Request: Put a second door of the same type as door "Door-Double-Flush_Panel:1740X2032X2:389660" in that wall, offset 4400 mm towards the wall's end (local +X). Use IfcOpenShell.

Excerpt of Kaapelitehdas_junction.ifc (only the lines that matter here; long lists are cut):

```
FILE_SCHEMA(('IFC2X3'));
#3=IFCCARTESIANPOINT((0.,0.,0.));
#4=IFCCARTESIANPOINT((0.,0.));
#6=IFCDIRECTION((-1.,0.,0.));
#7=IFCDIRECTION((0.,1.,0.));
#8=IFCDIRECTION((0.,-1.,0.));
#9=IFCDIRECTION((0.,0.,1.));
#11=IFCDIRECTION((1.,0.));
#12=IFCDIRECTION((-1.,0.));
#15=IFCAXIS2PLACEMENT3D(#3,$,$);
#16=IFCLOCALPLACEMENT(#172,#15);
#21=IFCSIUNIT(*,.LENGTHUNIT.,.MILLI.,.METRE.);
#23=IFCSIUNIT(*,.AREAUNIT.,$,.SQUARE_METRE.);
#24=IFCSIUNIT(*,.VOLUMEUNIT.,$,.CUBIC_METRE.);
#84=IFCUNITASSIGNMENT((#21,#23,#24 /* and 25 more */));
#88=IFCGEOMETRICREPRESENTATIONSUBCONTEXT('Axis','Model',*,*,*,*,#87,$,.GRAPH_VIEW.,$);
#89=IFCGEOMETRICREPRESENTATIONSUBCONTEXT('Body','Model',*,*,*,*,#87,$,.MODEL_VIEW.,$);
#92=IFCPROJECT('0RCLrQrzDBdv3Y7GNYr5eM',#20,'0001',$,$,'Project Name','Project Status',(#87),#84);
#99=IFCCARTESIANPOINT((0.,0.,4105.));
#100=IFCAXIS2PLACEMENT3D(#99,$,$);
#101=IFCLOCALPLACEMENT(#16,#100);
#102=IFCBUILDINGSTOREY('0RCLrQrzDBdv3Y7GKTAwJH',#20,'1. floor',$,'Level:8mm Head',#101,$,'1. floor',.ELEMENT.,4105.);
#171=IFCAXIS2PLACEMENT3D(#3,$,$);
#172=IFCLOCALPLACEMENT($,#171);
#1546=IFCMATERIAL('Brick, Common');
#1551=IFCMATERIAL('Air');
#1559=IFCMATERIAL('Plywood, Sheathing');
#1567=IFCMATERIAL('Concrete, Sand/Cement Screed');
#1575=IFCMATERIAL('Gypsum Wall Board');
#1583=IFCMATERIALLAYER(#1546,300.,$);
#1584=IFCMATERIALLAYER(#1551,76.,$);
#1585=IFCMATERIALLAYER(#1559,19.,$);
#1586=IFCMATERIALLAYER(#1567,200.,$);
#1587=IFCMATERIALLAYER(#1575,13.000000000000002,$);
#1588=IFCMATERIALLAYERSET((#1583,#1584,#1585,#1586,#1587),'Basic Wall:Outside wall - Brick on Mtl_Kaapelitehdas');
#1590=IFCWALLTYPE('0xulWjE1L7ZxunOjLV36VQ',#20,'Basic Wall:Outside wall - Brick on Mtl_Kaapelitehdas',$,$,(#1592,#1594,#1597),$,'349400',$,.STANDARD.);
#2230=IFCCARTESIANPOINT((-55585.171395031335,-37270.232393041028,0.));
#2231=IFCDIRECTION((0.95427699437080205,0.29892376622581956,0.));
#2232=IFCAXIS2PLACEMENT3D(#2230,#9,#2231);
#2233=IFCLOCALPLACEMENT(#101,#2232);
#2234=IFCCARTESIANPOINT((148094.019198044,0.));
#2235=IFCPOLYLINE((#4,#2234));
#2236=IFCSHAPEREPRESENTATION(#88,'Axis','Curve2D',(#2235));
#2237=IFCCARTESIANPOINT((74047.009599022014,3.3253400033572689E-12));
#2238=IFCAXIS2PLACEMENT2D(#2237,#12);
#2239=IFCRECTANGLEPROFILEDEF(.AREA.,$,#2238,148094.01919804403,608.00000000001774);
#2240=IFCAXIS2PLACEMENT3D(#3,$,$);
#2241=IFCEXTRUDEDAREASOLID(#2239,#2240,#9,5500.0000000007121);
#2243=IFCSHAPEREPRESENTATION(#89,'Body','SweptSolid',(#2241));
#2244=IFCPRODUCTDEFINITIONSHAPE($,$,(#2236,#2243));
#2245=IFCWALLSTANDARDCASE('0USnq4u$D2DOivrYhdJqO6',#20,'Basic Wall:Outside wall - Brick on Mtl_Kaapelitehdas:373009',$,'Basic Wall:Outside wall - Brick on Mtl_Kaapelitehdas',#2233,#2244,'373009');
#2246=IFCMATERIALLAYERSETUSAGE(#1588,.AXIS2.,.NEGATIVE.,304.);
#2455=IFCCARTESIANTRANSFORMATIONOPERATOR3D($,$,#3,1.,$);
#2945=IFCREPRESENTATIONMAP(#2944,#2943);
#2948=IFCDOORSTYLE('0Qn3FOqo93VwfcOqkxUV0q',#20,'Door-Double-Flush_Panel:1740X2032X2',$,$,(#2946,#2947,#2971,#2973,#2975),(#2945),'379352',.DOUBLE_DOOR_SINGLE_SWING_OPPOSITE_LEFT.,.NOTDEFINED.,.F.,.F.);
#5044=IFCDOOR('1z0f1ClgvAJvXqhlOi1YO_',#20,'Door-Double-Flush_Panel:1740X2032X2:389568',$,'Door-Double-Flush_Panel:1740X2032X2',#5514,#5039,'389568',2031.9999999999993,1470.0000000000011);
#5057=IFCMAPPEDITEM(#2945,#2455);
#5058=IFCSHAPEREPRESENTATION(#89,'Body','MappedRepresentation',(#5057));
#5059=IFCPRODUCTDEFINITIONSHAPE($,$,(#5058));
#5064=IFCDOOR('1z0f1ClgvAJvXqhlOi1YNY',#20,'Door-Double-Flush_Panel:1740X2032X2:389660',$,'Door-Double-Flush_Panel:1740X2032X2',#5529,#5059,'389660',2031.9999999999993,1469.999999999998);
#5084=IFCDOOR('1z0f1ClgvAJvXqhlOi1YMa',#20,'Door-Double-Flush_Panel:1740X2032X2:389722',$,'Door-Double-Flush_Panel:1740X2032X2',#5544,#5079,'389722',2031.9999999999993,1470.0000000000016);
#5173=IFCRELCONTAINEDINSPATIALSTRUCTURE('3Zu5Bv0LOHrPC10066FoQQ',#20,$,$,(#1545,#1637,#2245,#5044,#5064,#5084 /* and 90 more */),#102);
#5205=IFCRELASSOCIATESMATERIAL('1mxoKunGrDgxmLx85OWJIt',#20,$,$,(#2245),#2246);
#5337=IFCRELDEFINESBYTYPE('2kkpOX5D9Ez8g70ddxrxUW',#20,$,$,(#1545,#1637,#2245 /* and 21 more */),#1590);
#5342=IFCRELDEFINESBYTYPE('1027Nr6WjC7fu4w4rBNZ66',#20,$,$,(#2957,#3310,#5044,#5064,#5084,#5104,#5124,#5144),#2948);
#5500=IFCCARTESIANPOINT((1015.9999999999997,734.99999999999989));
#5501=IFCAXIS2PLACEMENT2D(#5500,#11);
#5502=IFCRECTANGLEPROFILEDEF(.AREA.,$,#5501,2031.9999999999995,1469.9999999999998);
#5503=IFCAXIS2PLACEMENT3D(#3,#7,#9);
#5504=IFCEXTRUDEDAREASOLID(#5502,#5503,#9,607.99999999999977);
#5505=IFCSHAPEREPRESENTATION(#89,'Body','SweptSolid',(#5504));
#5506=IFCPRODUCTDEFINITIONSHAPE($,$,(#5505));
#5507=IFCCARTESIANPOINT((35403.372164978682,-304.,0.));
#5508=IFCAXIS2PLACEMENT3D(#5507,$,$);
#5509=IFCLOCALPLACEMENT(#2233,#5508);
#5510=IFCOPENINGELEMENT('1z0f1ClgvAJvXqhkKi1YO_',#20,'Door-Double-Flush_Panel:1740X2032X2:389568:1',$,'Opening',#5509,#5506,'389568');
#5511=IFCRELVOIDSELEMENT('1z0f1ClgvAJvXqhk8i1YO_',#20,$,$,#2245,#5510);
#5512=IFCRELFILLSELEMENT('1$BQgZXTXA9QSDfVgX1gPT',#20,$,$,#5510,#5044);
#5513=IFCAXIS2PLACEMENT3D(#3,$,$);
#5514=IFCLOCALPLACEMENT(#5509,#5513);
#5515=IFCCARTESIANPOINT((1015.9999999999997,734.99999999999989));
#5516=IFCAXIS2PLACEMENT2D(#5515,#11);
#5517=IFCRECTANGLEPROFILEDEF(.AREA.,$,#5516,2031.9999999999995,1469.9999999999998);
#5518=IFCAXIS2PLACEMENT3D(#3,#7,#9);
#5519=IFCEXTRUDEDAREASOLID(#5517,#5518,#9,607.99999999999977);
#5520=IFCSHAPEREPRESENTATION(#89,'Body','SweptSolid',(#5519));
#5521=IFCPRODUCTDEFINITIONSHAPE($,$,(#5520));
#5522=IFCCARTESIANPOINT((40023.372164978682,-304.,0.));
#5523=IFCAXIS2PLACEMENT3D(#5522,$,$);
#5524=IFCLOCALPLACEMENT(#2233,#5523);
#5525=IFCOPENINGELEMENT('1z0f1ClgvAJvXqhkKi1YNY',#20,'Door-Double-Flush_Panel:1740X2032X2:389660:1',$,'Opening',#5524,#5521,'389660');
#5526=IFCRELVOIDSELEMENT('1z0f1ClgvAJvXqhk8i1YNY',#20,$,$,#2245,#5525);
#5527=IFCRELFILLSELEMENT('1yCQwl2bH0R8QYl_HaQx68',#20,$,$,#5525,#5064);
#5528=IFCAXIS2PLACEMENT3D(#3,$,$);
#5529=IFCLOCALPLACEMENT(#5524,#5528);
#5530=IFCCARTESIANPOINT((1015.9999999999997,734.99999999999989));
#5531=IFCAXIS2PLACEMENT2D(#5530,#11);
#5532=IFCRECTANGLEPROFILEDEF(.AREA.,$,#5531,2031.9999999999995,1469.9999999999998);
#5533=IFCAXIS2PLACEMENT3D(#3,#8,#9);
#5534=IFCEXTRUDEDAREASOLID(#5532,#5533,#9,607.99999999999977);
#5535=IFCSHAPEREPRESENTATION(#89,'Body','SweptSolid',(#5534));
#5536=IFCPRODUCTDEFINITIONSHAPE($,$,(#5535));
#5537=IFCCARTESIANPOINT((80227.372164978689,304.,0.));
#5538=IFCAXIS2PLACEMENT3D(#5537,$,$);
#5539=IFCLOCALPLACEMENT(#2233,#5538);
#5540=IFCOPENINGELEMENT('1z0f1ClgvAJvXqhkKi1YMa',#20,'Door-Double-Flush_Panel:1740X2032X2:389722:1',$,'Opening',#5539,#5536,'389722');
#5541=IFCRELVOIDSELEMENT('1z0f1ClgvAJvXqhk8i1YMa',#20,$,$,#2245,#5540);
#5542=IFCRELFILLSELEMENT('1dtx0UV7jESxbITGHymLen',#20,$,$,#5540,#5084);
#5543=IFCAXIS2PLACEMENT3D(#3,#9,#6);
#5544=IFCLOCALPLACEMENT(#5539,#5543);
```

```python
import ifcopenshell
import ifcopenshell.api.feature
import ifcopenshell.api.geometry
import ifcopenshell.api.root
import ifcopenshell.geom
import ifcopenshell.util.element
import ifcopenshell.util.placement
import ifcopenshell.util.shape

model = ifcopenshell.open("Kaapelitehdas_junction.ifc")
settings = ifcopenshell.geom.settings()


def volume(element):
    """Net volume in cubic metres, openings subtracted."""
    shape = ifcopenshell.geom.create_shape(settings, element)
    return ifcopenshell.util.shape.get_volume(shape.geometry)


def reuse_history(source, copy):
    """copy_class also copies each property set's owner history, people and application; keep the originals."""
    for rel in copy.IsDefinedBy:
        if rel.is_a("IfcRelDefinesByProperties") and (history := rel.RelatingPropertyDefinition.OwnerHistory):
            rel.RelatingPropertyDefinition.OwnerHistory = source.OwnerHistory
            ifcopenshell.util.element.remove_deep2(model, history)


door = model.by_id(5064)
opening = door.FillsVoids[0].RelatingOpeningElement
wall = opening.VoidsElements[0].RelatingBuildingElement
before = volume(wall)
shift = ifcopenshell.util.placement.get_local_placement(wall.ObjectPlacement)[:3, 0] * 4400.0

# copy_class copies the void relationship, type, container and properties, but no geometry.
new_opening = ifcopenshell.api.root.copy_class(model, product=opening)
new_opening.Representation = ifcopenshell.util.element.copy_deep(
    model, opening.Representation, exclude=["IfcGeometricRepresentationContext", "IfcRepresentationMap"]
)
new_opening.Name = "Door-Double-Flush_Panel:1740X2032X2"
new_opening.Tag = None
new_door = ifcopenshell.api.root.copy_class(model, product=door)
new_door.Representation = ifcopenshell.util.element.copy_deep(
    model, door.Representation, exclude=["IfcGeometricRepresentationContext", "IfcRepresentationMap"]
)
new_door.Name = "Door-Double-Flush_Panel:1740X2032X2"
new_door.Tag = None
reuse_history(door, new_door)
fills = ifcopenshell.api.feature.add_filling(model, opening=new_opening, element=new_door)
fills.OwnerHistory = new_door.OwnerHistory  # required in IFC2X3

for old, new in ((opening, new_opening), (door, new_door)):
    matrix = ifcopenshell.util.placement.get_local_placement(old.ObjectPlacement)
    matrix[:3, 3] += shift
    ifcopenshell.api.geometry.edit_object_placement(model, product=new, matrix=matrix, is_si=False)

after = volume(wall)

print(f"wall volume {before:.3f} -> {after:.3f} m3")

model.write("Kaapelitehdas_junction_v2.ifc")
```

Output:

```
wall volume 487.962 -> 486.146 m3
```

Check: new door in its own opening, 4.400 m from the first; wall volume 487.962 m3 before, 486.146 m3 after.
